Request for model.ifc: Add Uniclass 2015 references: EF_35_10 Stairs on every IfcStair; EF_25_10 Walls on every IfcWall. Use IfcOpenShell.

First a look at what the model holds.

```python
import ifcopenshell

model = ifcopenshell.open("model.ifc")
print(model.schema)
print("classifications:", [c.Name for c in model.by_type("IfcClassification")])
for ifc_class in ("IfcDoor", "IfcRoof", "IfcStair", "IfcWall", "IfcWindow"):
    print(ifc_class, len(model.by_type(ifc_class)))
```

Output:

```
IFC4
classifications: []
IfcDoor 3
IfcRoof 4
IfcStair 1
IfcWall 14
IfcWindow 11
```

```python
import ifcopenshell
import ifcopenshell.api.classification

model = ifcopenshell.open("model.ifc")

system = ifcopenshell.api.classification.add_classification(model, classification="Uniclass 2015")

codes = {
    "IfcStair": ("EF_35_10", "Stairs"),
    "IfcWall": ("EF_25_10", "Walls"),
}
for ifc_class, (code, name) in codes.items():
    products = model.by_type(ifc_class)
    ifcopenshell.api.classification.add_reference(
        model, products=products, classification=system, identification=code, name=name
    )
    print(code, len(products))

model.write("model_v2.ifc")
```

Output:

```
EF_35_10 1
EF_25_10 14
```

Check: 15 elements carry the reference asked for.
